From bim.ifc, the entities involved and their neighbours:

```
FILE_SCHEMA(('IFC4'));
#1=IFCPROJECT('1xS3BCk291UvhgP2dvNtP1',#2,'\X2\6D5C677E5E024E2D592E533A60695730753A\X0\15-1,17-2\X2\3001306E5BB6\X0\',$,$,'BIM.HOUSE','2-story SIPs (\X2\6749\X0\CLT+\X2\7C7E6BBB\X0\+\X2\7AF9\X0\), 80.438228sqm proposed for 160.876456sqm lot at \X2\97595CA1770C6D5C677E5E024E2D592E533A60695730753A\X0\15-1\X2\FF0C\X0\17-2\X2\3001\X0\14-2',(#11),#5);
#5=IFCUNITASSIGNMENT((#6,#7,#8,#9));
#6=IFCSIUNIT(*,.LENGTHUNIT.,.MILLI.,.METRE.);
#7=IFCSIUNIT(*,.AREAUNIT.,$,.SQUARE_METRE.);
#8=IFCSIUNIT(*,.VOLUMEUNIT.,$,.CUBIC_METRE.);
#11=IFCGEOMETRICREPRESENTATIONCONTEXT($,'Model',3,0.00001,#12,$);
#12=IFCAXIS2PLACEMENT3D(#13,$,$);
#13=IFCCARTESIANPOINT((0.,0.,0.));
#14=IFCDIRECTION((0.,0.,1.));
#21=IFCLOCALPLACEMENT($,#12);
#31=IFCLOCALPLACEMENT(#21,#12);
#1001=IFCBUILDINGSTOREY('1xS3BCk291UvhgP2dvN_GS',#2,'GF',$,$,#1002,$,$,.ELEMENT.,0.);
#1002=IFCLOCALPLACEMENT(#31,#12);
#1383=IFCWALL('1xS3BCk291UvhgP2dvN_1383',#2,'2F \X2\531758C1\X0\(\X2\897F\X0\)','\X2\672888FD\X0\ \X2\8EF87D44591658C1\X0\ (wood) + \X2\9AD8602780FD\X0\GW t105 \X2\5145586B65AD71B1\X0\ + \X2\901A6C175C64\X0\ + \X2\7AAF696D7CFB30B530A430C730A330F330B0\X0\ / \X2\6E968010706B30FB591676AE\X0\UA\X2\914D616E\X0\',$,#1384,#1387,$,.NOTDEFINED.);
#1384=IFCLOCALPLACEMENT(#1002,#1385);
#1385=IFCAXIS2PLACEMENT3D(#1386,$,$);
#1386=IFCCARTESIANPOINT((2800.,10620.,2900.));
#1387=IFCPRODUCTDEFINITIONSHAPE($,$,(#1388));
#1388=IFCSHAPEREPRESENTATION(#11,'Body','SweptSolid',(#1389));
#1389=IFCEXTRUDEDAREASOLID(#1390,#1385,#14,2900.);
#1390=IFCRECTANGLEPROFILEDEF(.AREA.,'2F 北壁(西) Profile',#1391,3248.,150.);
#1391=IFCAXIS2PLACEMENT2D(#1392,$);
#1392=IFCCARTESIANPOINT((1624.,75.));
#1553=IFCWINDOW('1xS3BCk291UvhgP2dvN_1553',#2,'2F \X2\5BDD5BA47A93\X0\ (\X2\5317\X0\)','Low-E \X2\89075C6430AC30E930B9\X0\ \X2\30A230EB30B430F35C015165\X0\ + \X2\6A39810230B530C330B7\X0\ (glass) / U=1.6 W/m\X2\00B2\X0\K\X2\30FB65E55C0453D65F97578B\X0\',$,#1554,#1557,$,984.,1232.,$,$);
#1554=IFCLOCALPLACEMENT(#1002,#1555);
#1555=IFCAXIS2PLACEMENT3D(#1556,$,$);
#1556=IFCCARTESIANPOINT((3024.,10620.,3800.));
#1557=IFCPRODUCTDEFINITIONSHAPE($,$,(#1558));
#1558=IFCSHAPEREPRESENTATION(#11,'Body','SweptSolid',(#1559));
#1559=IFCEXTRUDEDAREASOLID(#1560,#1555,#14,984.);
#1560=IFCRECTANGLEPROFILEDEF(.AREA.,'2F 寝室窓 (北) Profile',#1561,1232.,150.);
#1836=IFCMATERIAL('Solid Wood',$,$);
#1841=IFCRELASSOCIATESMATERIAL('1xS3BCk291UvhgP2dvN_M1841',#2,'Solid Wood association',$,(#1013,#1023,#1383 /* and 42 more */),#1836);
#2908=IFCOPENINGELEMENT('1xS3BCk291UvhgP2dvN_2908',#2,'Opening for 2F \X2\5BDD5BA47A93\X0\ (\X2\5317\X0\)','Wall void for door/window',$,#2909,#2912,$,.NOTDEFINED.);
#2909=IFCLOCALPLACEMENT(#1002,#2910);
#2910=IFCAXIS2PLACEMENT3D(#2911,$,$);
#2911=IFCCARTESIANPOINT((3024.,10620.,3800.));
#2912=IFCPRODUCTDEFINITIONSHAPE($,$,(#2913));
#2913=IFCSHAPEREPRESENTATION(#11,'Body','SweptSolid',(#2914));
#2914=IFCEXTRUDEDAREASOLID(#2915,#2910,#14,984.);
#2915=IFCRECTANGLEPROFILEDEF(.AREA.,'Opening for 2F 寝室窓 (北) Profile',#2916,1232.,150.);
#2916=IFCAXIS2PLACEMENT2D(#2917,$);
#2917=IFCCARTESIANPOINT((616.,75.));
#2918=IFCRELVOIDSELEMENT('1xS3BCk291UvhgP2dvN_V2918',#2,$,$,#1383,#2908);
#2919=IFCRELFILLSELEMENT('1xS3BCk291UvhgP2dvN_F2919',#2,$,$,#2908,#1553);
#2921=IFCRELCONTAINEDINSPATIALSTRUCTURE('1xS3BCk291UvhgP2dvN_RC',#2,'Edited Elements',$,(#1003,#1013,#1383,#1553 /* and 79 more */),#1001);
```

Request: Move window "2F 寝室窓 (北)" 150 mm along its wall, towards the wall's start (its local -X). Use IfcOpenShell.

```python
import ifcopenshell
import ifcopenshell.api.geometry
import ifcopenshell.util.placement

model = ifcopenshell.open("bim.ifc")

window = model.by_guid("1xS3BCk291UvhgP2dvN_1553")
opening = window.FillsVoids[0].RelatingOpeningElement
wall = opening.VoidsElements[0].RelatingBuildingElement

wall_matrix = ifcopenshell.util.placement.get_local_placement(wall.ObjectPlacement)
shift = wall_matrix[:3, 0] * -150.0
before = ifcopenshell.util.placement.get_local_placement(window.ObjectPlacement)[:3, 3].copy()

# The window is not placed relative to its opening, so move both.
for product in (opening, window):
    matrix = ifcopenshell.util.placement.get_local_placement(product.ObjectPlacement)
    matrix[:3, 3] += shift
    ifcopenshell.api.geometry.edit_object_placement(model, product=product, matrix=matrix, is_si=False)

after = ifcopenshell.util.placement.get_local_placement(window.ObjectPlacement)[:3, 3]
print("window moved by", (after - before).round(3) + 0.0)

model.write("bim-out.ifc")
```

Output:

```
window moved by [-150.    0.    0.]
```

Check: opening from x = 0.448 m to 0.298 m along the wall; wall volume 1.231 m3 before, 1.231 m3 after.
